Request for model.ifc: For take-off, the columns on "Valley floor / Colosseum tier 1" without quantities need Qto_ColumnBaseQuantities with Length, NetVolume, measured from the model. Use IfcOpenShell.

First a look at what the model holds.

```python
import ifcopenshell
import ifcopenshell.util.element
import ifcopenshell.util.unit

model = ifcopenshell.open("model.ifc")
print(model.schema)
for unit_type in ("LENGTHUNIT", "AREAUNIT", "VOLUMEUNIT"):
    print(unit_type, ifcopenshell.util.unit.calculate_unit_scale(model, unit_type))
storey = next(s for s in model.by_type("IfcBuildingStorey") if s.Name == "Valley floor / Colosseum tier 1")
columns = [e for e in ifcopenshell.util.element.get_decomposition(storey) if e.is_a("IfcColumn")]
for e in sorted(columns, key=lambda e: e.id()):
    print(e.id(), e.is_a(), e.Name, list(ifcopenshell.util.element.get_psets(e, qtos_only=True)), sep=" | ")
```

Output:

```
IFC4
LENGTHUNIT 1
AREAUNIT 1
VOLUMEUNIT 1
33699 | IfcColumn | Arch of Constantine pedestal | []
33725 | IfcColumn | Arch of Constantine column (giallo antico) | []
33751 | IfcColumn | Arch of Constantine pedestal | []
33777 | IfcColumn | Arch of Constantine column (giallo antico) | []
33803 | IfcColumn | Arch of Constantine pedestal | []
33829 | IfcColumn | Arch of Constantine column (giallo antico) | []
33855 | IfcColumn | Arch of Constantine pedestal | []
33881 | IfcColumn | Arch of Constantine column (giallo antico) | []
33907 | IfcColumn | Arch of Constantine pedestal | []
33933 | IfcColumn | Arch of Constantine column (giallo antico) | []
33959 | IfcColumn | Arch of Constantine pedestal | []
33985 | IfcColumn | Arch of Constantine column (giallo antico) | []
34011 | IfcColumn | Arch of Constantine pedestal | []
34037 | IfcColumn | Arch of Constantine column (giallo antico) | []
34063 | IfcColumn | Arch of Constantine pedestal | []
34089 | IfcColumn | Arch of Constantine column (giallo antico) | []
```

```python
import ifcopenshell
import ifcopenshell.api.pset
import ifcopenshell.geom
import ifcopenshell.util.element
import ifcopenshell.util.shape
import ifcopenshell.util.unit

model = ifcopenshell.open("model.ifc")
unit_scale = ifcopenshell.util.unit.calculate_unit_scale(model)
volume_scale = ifcopenshell.util.unit.calculate_unit_scale(model, "VOLUMEUNIT")
settings = ifcopenshell.geom.settings()

storey = next(s for s in model.by_type("IfcBuildingStorey") if s.Name == "Valley floor / Colosseum tier 1")
columns = [e for e in ifcopenshell.util.element.get_decomposition(storey) if e.is_a("IfcColumn")]

for e in sorted(columns, key=lambda e: e.id()):
    if ifcopenshell.util.element.get_psets(e, qtos_only=True, should_inherit=False):
        continue
    # Geometry comes back in metres, in the element's own axes.
    shape = ifcopenshell.geom.create_shape(settings, e)
    values = {
        "Length": ifcopenshell.util.shape.get_z(shape.geometry) / unit_scale,
        "NetVolume": ifcopenshell.util.shape.get_volume(shape.geometry) / volume_scale,
    }
    qto = ifcopenshell.api.pset.add_qto(model, product=e, name="Qto_ColumnBaseQuantities")
    ifcopenshell.api.pset.edit_qto(model, qto=qto, properties=values)
    print(e.id(), {k: round(v, 3) for k, v in values.items()})

model.write("model_edited.ifc")
```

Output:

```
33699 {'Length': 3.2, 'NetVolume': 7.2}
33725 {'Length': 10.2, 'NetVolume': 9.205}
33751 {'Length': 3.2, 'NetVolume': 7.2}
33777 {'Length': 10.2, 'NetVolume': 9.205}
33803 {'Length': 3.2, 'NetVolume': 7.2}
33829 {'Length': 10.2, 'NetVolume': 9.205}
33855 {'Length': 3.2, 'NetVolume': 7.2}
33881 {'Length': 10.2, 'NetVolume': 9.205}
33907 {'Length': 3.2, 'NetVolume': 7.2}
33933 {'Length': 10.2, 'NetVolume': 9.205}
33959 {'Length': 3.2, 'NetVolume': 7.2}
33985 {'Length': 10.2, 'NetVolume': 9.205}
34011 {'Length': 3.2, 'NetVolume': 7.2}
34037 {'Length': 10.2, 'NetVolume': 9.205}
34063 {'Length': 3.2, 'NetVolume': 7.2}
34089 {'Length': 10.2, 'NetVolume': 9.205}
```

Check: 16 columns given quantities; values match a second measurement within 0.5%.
